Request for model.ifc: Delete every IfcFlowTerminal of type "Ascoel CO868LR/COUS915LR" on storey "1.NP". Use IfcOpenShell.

First a look at what the model holds.

```python
import ifcopenshell
import ifcopenshell.util.element

model = ifcopenshell.open("model.ifc")
print(model.schema)
storey = next(s for s in model.by_type("IfcBuildingStorey") if s.Name == "1.NP")
terminals = [e for e in ifcopenshell.util.element.get_decomposition(storey) if e.is_a("IfcFlowTerminal")]
seen = {}
for e in terminals:
    element_type = ifcopenshell.util.element.get_type(e)
    name = element_type.Name if element_type not in (None, e) else None
    seen[name] = seen.get(name, 0) + 1
for name, count in sorted(seen.items(), key=str):
    print(count, "x", name)
```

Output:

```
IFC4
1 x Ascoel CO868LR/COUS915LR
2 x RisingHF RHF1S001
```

```python
import ifcopenshell
import ifcopenshell.api.root
import ifcopenshell.util.element

model = ifcopenshell.open("model.ifc")

storey = next(s for s in model.by_type("IfcBuildingStorey") if s.Name == "1.NP")
terminals = [e for e in ifcopenshell.util.element.get_decomposition(storey) if e.is_a("IfcFlowTerminal")]
targets = [e for e in terminals if (t := ifcopenshell.util.element.get_type(e)) not in (None, e) and t.Name == "Ascoel CO868LR/COUS915LR"]

for e in targets:
    ifcopenshell.api.root.remove_product(model, product=e)
print(len(targets), "removed")

model.write("model_updated.ifc")
```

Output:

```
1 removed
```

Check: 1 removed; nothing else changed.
